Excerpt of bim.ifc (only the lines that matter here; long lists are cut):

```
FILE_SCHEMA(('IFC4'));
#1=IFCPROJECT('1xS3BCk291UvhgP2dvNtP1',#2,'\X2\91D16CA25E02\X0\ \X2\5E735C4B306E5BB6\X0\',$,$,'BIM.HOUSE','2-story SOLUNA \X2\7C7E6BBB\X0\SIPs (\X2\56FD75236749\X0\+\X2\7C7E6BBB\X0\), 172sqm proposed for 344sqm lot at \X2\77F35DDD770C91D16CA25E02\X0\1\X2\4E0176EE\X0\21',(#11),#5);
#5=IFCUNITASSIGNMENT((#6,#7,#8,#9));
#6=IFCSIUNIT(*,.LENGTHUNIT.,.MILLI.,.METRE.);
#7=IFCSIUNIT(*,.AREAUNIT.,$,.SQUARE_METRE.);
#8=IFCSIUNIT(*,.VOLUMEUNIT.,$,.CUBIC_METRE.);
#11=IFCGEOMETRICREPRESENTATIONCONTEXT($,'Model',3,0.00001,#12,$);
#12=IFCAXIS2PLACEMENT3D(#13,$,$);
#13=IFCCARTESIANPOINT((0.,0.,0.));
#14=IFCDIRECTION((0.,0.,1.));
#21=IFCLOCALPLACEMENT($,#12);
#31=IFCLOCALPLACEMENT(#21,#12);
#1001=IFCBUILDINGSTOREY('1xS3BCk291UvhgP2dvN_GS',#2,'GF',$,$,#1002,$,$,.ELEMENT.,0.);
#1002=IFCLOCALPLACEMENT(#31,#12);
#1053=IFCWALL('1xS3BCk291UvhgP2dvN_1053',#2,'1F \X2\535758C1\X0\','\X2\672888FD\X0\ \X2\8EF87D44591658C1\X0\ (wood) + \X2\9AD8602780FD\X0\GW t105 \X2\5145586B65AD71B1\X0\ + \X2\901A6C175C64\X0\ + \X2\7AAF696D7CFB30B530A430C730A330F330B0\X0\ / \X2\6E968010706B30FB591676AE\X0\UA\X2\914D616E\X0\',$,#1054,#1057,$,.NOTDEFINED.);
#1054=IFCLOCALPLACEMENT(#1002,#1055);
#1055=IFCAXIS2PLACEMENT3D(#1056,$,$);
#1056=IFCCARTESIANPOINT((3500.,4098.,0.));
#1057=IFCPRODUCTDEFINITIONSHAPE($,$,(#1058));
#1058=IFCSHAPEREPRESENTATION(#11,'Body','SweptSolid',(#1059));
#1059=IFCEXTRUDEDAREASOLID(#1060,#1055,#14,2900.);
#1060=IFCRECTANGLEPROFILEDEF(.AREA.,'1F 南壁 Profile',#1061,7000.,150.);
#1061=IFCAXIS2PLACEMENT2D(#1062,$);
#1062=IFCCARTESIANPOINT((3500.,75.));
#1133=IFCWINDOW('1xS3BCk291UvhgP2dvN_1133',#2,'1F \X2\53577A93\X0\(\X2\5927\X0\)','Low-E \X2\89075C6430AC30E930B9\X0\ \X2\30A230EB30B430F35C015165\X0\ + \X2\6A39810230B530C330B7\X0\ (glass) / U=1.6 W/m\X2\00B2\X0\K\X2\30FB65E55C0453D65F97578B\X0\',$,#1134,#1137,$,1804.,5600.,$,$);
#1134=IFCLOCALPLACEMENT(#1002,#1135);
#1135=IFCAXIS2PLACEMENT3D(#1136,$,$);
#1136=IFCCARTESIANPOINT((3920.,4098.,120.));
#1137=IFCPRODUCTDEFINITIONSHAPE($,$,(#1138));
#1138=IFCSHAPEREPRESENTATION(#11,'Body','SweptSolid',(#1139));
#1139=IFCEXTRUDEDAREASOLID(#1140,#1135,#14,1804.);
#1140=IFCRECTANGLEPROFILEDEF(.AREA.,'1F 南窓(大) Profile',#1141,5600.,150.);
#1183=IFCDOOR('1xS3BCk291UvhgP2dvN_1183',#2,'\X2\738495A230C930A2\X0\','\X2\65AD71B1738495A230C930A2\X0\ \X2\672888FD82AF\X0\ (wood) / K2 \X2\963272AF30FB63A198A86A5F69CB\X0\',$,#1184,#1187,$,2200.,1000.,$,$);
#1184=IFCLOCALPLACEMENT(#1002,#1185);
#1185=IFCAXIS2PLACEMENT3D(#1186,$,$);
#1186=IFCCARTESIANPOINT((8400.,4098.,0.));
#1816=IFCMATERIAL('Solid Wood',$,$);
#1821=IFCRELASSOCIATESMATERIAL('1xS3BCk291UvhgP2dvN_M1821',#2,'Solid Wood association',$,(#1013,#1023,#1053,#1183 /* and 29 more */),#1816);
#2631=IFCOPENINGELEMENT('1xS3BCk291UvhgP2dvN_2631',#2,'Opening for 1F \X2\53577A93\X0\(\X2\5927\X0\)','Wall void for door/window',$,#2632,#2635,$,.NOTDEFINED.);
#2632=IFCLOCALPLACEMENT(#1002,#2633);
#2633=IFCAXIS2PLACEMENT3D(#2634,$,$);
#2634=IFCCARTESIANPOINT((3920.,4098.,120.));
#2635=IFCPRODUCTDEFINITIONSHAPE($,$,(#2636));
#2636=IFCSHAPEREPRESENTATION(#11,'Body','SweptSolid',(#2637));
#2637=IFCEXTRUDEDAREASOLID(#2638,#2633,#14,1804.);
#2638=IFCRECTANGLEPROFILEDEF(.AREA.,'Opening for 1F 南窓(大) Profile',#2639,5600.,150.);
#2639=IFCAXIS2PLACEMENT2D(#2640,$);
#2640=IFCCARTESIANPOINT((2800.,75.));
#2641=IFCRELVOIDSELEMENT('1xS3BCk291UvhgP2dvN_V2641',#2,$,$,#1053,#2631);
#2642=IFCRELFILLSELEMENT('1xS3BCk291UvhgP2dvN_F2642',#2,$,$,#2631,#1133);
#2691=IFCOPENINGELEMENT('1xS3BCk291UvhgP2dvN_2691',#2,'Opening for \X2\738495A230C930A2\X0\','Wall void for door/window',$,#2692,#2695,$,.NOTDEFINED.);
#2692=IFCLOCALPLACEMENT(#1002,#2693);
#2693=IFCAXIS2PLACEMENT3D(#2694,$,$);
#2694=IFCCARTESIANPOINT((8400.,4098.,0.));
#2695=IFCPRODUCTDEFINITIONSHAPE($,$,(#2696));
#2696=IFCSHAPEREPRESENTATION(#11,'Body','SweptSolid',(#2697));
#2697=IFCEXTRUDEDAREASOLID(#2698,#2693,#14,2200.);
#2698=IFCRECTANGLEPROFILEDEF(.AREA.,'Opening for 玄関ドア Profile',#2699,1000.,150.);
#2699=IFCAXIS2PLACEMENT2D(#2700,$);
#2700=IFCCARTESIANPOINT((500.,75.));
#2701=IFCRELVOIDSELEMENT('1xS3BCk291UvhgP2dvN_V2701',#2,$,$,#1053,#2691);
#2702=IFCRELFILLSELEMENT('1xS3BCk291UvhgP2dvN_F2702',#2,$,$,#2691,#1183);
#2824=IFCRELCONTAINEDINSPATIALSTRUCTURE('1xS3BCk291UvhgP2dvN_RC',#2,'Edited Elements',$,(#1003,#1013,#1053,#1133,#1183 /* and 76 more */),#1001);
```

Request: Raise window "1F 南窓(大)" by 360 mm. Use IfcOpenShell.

```python
import numpy as np
import ifcopenshell
import ifcopenshell.api.geometry
import ifcopenshell.util.placement
import ifcopenshell.util.unit

model = ifcopenshell.open("bim.ifc")
unit_scale = ifcopenshell.util.unit.calculate_unit_scale(model)

window = model.by_id(1133)
opening = window.FillsVoids[0].RelatingOpeningElement
dz = 360.0

shift = np.array([0.0, 0.0, dz])
# The window is not placed relative to its opening, so move both.
for product in (opening, window):
    matrix = ifcopenshell.util.placement.get_local_placement(product.ObjectPlacement)
    matrix[:3, 3] += shift
    ifcopenshell.api.geometry.edit_object_placement(model, product=product, matrix=matrix, is_si=False)

print(f"moved by {dz * unit_scale:+.3f} m")

model.write("bim_updated.ifc")
```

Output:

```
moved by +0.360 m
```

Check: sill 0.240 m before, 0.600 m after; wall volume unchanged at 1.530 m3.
